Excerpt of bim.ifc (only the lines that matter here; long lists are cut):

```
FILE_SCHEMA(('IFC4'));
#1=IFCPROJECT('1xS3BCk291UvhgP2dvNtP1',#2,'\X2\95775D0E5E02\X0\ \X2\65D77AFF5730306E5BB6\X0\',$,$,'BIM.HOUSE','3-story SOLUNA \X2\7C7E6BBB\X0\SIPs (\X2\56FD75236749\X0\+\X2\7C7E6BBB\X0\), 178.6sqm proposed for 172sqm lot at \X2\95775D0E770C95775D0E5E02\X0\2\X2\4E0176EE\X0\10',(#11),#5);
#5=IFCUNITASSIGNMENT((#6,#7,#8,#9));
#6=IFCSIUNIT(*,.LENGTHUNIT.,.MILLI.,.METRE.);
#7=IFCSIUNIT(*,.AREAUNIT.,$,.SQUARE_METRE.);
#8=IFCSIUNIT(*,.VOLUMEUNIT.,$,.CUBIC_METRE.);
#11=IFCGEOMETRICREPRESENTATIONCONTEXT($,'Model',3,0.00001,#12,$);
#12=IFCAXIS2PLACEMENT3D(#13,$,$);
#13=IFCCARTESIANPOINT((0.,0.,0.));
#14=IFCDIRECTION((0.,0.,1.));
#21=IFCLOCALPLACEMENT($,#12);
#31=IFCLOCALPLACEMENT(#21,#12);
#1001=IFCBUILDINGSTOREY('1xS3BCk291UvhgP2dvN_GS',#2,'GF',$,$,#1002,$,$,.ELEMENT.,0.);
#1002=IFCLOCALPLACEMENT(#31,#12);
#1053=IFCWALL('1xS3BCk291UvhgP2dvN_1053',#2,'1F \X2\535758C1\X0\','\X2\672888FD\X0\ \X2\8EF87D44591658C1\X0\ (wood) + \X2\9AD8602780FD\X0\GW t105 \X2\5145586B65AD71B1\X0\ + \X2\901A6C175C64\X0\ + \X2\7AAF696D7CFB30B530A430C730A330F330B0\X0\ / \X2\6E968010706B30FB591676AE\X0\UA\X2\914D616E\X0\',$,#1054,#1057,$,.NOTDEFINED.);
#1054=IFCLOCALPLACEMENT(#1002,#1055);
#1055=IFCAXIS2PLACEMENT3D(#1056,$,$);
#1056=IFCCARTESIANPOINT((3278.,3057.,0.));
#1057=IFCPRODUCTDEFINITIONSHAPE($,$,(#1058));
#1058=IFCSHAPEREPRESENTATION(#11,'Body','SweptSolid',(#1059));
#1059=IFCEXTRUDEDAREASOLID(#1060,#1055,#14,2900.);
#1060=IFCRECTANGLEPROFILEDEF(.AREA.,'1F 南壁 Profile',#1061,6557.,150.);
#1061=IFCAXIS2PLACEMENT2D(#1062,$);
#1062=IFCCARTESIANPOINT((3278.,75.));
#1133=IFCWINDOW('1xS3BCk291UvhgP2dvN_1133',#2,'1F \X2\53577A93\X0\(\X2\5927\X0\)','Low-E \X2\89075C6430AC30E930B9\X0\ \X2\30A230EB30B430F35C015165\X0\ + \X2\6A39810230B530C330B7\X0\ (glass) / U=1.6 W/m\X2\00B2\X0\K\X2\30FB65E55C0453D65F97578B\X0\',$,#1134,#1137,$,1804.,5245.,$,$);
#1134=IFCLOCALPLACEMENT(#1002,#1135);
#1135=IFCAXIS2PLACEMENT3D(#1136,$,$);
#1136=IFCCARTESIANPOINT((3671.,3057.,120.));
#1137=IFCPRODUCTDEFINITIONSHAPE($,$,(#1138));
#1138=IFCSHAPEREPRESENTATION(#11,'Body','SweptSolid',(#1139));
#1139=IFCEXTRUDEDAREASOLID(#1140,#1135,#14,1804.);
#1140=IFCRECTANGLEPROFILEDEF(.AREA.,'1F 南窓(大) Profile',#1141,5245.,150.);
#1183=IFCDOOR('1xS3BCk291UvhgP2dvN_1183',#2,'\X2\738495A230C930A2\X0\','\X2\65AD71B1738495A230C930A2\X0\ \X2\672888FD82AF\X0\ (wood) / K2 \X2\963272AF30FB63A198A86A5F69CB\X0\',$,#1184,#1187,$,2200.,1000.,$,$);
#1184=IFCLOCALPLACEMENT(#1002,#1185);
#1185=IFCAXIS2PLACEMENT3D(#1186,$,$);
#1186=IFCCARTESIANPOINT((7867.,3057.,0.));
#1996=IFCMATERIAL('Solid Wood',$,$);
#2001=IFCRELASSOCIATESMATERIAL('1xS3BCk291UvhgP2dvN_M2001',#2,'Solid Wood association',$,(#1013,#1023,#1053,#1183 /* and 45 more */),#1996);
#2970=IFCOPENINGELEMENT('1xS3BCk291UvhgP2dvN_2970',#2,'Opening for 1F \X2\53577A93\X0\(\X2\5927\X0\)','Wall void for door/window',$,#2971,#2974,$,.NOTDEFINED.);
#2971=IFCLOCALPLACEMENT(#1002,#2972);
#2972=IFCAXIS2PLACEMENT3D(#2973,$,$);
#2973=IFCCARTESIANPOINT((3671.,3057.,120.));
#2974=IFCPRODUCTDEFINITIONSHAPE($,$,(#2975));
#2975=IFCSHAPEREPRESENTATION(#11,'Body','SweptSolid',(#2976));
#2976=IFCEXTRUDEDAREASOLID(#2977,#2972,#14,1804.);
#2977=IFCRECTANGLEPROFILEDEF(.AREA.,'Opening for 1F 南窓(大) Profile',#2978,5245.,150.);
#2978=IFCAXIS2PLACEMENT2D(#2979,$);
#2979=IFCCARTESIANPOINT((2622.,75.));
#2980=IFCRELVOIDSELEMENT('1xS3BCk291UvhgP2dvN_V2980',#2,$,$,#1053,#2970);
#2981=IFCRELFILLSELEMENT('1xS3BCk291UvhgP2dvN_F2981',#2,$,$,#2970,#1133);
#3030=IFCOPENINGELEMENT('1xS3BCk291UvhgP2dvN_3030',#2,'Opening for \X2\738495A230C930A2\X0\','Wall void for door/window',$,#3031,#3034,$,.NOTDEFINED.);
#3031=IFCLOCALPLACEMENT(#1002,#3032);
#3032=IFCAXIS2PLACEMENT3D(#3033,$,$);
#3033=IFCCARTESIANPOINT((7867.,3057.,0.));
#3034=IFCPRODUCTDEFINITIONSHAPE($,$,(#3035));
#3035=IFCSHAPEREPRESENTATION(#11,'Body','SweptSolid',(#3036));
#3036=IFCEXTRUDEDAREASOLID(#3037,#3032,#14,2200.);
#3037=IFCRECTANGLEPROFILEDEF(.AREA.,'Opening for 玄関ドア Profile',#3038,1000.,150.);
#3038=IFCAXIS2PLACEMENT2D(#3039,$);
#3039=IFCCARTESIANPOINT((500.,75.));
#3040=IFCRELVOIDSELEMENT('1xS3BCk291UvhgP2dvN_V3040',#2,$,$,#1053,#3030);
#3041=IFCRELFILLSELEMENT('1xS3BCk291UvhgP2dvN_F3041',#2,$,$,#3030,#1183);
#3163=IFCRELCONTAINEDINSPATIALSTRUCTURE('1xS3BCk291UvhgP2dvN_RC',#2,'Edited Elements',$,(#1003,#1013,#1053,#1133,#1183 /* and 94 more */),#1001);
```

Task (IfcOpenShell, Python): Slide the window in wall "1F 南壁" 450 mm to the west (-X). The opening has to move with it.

```python
import ifcopenshell
import ifcopenshell.api.geometry
import ifcopenshell.util.placement
import ifcopenshell.util.unit

model = ifcopenshell.open("bim.ifc")
unit_scale = ifcopenshell.util.unit.calculate_unit_scale(model)

window = model.by_guid("1xS3BCk291UvhgP2dvN_1133")
opening = window.FillsVoids[0].RelatingOpeningElement
wall = opening.VoidsElements[0].RelatingBuildingElement

wall_matrix = ifcopenshell.util.placement.get_local_placement(wall.ObjectPlacement)
shift = wall_matrix[:3, 0] * -0.45 / unit_scale
before = ifcopenshell.util.placement.get_local_placement(window.ObjectPlacement)[:3, 3].copy()

# The window is not placed relative to its opening, so move both.
for product in (opening, window):
    matrix = ifcopenshell.util.placement.get_local_placement(product.ObjectPlacement)
    matrix[:3, 3] += shift
    ifcopenshell.api.geometry.edit_object_placement(model, product=product, matrix=matrix, is_si=False)

after = ifcopenshell.util.placement.get_local_placement(window.ObjectPlacement)[:3, 3]
print("window moved by", (after - before).round(3) + 0.0)

model.write("bim_edited.ifc")
```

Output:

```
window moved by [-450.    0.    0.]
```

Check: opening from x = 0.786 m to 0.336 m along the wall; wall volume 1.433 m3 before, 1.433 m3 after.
